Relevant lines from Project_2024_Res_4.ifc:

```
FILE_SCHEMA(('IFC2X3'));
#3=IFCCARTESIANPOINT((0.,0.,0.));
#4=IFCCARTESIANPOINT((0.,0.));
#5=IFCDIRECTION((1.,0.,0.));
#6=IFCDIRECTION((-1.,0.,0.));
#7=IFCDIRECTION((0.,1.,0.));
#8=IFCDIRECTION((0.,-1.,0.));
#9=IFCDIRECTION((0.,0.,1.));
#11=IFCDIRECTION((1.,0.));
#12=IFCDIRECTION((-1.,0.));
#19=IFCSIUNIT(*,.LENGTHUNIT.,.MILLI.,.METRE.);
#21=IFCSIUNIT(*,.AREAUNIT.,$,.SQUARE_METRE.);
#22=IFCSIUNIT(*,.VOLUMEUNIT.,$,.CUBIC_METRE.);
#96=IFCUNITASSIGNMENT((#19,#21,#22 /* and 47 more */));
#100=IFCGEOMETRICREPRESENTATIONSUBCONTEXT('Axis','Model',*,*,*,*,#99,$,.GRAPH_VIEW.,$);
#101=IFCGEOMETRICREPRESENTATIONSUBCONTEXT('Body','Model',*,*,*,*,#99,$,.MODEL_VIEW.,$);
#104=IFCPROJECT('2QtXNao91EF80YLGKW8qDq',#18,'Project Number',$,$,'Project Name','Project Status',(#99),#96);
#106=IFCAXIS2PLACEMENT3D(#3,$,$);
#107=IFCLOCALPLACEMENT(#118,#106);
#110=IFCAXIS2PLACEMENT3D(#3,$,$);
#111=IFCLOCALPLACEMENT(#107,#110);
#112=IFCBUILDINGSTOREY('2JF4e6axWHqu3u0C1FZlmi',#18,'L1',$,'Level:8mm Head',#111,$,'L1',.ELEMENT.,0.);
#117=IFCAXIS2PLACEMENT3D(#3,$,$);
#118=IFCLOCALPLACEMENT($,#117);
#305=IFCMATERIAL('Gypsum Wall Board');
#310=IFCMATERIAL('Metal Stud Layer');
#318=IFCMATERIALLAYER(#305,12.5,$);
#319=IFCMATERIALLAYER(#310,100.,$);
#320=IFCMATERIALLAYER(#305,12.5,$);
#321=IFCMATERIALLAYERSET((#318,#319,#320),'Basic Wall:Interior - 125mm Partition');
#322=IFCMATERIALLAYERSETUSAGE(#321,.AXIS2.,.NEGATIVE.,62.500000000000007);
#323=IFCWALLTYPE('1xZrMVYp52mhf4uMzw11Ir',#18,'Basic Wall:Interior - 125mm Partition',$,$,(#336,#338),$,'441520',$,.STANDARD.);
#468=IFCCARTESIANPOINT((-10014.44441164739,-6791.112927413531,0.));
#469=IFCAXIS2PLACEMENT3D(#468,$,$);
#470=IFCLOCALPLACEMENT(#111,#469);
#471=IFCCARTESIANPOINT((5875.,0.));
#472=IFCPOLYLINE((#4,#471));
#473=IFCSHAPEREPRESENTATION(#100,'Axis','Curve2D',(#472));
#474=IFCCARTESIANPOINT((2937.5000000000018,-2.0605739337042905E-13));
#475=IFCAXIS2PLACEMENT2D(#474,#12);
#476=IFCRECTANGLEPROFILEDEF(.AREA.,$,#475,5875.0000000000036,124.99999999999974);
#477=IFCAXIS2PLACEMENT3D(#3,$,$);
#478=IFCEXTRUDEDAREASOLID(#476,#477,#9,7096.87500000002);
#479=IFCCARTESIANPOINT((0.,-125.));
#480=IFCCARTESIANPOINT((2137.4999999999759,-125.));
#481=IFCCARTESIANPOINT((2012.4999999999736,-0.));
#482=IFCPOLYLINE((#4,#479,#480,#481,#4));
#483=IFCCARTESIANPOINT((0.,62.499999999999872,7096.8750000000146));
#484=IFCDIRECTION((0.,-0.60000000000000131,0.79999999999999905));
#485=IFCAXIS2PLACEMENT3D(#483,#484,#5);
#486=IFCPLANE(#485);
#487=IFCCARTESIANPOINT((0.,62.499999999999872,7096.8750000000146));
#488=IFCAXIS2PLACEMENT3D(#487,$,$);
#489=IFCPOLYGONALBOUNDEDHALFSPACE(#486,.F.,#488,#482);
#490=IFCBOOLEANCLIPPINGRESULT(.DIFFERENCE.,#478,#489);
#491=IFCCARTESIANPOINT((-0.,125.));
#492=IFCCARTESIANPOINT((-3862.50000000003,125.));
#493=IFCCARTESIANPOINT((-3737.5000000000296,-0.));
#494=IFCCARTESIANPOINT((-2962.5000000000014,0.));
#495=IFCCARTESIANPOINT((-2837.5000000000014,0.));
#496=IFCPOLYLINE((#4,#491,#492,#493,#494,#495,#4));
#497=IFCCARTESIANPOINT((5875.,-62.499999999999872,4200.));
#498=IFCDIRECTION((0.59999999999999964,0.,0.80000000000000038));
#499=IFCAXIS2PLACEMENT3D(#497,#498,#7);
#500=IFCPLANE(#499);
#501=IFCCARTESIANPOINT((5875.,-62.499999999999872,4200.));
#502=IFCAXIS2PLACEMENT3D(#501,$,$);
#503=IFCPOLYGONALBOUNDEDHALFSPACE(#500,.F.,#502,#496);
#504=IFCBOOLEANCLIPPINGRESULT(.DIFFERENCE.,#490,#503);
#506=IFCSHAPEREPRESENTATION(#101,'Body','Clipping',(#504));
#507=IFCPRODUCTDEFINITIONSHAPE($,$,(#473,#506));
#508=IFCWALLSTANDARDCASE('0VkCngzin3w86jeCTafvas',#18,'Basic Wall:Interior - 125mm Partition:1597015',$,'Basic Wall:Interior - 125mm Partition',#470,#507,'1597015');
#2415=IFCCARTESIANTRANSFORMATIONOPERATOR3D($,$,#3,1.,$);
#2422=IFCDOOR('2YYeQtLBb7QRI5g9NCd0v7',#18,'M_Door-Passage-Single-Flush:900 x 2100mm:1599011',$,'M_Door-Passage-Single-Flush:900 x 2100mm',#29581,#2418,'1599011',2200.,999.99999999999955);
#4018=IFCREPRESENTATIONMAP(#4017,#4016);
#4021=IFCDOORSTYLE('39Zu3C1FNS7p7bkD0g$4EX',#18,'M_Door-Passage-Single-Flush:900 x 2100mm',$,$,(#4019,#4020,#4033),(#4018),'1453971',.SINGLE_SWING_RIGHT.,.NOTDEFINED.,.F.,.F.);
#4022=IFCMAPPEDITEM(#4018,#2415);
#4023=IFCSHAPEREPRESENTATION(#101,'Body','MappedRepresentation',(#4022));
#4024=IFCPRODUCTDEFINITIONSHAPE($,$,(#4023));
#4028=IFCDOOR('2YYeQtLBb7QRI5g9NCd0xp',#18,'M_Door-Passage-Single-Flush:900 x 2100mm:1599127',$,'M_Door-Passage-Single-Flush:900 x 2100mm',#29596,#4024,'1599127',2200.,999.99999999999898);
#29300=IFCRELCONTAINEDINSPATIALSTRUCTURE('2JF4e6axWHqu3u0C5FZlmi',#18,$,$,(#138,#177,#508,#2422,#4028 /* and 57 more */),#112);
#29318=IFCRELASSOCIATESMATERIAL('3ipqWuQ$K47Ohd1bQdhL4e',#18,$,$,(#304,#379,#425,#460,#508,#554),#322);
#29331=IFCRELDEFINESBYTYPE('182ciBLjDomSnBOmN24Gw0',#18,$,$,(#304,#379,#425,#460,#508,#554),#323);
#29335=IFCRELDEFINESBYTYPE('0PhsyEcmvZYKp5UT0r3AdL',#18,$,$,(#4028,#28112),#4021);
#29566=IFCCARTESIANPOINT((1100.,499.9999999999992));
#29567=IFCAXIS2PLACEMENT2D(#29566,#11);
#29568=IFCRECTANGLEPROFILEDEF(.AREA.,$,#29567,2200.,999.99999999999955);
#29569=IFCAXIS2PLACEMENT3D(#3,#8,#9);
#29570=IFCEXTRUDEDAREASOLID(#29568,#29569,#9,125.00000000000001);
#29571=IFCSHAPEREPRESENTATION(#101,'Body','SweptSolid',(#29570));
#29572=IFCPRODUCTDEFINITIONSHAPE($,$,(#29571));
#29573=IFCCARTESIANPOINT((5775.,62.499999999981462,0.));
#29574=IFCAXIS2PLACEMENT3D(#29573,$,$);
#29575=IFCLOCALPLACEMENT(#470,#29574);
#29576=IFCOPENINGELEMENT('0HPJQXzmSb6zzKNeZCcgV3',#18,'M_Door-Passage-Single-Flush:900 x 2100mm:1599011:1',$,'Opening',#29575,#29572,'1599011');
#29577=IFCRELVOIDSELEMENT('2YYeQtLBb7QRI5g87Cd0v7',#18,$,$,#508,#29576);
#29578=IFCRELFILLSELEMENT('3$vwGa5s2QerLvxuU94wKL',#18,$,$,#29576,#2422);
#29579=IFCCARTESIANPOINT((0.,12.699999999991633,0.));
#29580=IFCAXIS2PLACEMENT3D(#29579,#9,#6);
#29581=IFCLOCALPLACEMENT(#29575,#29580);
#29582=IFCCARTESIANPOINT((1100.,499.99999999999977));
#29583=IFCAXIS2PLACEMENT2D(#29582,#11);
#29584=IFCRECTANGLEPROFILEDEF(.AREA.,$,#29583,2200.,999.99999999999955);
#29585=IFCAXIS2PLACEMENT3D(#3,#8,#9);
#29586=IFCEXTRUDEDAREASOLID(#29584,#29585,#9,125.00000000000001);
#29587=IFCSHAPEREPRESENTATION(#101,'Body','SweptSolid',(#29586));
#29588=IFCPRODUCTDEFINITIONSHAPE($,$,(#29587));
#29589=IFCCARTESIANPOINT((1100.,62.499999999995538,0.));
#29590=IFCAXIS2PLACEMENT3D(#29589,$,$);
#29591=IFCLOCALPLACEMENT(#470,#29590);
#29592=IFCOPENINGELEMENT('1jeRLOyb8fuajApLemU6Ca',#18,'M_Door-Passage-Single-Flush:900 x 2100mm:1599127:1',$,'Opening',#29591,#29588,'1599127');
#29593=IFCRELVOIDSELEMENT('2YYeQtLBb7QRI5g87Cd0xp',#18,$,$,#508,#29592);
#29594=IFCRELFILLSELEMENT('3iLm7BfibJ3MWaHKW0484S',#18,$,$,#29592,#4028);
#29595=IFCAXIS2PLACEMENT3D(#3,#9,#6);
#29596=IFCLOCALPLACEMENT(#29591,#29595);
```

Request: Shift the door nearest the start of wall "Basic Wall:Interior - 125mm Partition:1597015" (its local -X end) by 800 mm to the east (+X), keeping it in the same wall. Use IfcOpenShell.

```python
import ifcopenshell
import ifcopenshell.api.geometry
import ifcopenshell.util.placement
import ifcopenshell.util.unit

model = ifcopenshell.open("Project_2024_Res_4.ifc")
unit_scale = ifcopenshell.util.unit.calculate_unit_scale(model)

door = model.by_guid("2YYeQtLBb7QRI5g9NCd0xp")
opening = door.FillsVoids[0].RelatingOpeningElement
wall = opening.VoidsElements[0].RelatingBuildingElement

wall_matrix = ifcopenshell.util.placement.get_local_placement(wall.ObjectPlacement)
shift = wall_matrix[:3, 0] * 0.8 / unit_scale
before = ifcopenshell.util.placement.get_local_placement(door.ObjectPlacement)[:3, 3].copy()

# The door is placed relative to its opening, so it follows when the opening moves.
matrix = ifcopenshell.util.placement.get_local_placement(opening.ObjectPlacement)
matrix[:3, 3] += shift
ifcopenshell.api.geometry.edit_object_placement(
    model, product=opening, matrix=matrix, is_si=False, should_transform_children=True
)

after = ifcopenshell.util.placement.get_local_placement(door.ObjectPlacement)[:3, 3]
print("door moved by", (after - before).round(3) + 0.0)

model.write("Project_2024_Res_4_rev.ifc")
```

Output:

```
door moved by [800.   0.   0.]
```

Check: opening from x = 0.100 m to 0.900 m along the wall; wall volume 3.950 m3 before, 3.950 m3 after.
